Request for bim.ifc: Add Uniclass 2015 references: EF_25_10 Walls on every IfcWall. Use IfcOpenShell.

First a look at what the model holds.

```python
import ifcopenshell

model = ifcopenshell.open("bim.ifc")
print(model.schema)
print("classifications:", [c.Name for c in model.by_type("IfcClassification")])
for ifc_class in ("IfcDoor", "IfcRoof", "IfcStair", "IfcWall", "IfcWindow"):
    print(ifc_class, len(model.by_type(ifc_class)))
```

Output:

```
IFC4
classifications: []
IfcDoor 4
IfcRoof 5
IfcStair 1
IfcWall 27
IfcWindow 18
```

```python
import ifcopenshell
import ifcopenshell.api.classification

model = ifcopenshell.open("bim.ifc")

system = ifcopenshell.api.classification.add_classification(model, classification="Uniclass 2015")

codes = {
    "IfcWall": ("EF_25_10", "Walls"),
}
for ifc_class, (code, name) in codes.items():
    products = model.by_type(ifc_class)
    ifcopenshell.api.classification.add_reference(
        model, products=products, classification=system, identification=code, name=name
    )
    print(code, len(products))

model.write("bim_v2.ifc")
```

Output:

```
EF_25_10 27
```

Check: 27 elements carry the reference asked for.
